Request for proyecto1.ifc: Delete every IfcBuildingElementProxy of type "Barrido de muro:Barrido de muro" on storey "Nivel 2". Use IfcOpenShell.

First a look at what the model holds.

```python
import ifcopenshell
import ifcopenshell.util.element

model = ifcopenshell.open("proyecto1.ifc")
print(model.schema)
storey = next(s for s in model.by_type("IfcBuildingStorey") if s.Name == "Nivel 2")
proxies = [e for e in ifcopenshell.util.element.get_decomposition(storey) if e.is_a("IfcBuildingElementProxy")]
seen = {}
for e in proxies:
    element_type = ifcopenshell.util.element.get_type(e)
    name = element_type.Name if element_type not in (None, e) else None
    seen[name] = seen.get(name, 0) + 1
for name, count in sorted(seen.items(), key=str):
    print(count, "x", name)
```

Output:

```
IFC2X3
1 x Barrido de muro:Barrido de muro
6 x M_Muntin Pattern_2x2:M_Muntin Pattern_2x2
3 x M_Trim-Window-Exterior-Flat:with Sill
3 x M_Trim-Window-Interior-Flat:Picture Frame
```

```python
import ifcopenshell
import ifcopenshell.api.root
import ifcopenshell.util.element

model = ifcopenshell.open("proyecto1.ifc")

storey = next(s for s in model.by_type("IfcBuildingStorey") if s.Name == "Nivel 2")
proxies = [e for e in ifcopenshell.util.element.get_decomposition(storey) if e.is_a("IfcBuildingElementProxy")]
targets = [e for e in proxies if (t := ifcopenshell.util.element.get_type(e)) not in (None, e) and t.Name == "Barrido de muro:Barrido de muro"]

for e in targets:
    ifcopenshell.api.root.remove_product(model, product=e)
print(len(targets), "removed")

model.write("proyecto1_rev.ifc")
```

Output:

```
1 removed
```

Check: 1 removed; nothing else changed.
